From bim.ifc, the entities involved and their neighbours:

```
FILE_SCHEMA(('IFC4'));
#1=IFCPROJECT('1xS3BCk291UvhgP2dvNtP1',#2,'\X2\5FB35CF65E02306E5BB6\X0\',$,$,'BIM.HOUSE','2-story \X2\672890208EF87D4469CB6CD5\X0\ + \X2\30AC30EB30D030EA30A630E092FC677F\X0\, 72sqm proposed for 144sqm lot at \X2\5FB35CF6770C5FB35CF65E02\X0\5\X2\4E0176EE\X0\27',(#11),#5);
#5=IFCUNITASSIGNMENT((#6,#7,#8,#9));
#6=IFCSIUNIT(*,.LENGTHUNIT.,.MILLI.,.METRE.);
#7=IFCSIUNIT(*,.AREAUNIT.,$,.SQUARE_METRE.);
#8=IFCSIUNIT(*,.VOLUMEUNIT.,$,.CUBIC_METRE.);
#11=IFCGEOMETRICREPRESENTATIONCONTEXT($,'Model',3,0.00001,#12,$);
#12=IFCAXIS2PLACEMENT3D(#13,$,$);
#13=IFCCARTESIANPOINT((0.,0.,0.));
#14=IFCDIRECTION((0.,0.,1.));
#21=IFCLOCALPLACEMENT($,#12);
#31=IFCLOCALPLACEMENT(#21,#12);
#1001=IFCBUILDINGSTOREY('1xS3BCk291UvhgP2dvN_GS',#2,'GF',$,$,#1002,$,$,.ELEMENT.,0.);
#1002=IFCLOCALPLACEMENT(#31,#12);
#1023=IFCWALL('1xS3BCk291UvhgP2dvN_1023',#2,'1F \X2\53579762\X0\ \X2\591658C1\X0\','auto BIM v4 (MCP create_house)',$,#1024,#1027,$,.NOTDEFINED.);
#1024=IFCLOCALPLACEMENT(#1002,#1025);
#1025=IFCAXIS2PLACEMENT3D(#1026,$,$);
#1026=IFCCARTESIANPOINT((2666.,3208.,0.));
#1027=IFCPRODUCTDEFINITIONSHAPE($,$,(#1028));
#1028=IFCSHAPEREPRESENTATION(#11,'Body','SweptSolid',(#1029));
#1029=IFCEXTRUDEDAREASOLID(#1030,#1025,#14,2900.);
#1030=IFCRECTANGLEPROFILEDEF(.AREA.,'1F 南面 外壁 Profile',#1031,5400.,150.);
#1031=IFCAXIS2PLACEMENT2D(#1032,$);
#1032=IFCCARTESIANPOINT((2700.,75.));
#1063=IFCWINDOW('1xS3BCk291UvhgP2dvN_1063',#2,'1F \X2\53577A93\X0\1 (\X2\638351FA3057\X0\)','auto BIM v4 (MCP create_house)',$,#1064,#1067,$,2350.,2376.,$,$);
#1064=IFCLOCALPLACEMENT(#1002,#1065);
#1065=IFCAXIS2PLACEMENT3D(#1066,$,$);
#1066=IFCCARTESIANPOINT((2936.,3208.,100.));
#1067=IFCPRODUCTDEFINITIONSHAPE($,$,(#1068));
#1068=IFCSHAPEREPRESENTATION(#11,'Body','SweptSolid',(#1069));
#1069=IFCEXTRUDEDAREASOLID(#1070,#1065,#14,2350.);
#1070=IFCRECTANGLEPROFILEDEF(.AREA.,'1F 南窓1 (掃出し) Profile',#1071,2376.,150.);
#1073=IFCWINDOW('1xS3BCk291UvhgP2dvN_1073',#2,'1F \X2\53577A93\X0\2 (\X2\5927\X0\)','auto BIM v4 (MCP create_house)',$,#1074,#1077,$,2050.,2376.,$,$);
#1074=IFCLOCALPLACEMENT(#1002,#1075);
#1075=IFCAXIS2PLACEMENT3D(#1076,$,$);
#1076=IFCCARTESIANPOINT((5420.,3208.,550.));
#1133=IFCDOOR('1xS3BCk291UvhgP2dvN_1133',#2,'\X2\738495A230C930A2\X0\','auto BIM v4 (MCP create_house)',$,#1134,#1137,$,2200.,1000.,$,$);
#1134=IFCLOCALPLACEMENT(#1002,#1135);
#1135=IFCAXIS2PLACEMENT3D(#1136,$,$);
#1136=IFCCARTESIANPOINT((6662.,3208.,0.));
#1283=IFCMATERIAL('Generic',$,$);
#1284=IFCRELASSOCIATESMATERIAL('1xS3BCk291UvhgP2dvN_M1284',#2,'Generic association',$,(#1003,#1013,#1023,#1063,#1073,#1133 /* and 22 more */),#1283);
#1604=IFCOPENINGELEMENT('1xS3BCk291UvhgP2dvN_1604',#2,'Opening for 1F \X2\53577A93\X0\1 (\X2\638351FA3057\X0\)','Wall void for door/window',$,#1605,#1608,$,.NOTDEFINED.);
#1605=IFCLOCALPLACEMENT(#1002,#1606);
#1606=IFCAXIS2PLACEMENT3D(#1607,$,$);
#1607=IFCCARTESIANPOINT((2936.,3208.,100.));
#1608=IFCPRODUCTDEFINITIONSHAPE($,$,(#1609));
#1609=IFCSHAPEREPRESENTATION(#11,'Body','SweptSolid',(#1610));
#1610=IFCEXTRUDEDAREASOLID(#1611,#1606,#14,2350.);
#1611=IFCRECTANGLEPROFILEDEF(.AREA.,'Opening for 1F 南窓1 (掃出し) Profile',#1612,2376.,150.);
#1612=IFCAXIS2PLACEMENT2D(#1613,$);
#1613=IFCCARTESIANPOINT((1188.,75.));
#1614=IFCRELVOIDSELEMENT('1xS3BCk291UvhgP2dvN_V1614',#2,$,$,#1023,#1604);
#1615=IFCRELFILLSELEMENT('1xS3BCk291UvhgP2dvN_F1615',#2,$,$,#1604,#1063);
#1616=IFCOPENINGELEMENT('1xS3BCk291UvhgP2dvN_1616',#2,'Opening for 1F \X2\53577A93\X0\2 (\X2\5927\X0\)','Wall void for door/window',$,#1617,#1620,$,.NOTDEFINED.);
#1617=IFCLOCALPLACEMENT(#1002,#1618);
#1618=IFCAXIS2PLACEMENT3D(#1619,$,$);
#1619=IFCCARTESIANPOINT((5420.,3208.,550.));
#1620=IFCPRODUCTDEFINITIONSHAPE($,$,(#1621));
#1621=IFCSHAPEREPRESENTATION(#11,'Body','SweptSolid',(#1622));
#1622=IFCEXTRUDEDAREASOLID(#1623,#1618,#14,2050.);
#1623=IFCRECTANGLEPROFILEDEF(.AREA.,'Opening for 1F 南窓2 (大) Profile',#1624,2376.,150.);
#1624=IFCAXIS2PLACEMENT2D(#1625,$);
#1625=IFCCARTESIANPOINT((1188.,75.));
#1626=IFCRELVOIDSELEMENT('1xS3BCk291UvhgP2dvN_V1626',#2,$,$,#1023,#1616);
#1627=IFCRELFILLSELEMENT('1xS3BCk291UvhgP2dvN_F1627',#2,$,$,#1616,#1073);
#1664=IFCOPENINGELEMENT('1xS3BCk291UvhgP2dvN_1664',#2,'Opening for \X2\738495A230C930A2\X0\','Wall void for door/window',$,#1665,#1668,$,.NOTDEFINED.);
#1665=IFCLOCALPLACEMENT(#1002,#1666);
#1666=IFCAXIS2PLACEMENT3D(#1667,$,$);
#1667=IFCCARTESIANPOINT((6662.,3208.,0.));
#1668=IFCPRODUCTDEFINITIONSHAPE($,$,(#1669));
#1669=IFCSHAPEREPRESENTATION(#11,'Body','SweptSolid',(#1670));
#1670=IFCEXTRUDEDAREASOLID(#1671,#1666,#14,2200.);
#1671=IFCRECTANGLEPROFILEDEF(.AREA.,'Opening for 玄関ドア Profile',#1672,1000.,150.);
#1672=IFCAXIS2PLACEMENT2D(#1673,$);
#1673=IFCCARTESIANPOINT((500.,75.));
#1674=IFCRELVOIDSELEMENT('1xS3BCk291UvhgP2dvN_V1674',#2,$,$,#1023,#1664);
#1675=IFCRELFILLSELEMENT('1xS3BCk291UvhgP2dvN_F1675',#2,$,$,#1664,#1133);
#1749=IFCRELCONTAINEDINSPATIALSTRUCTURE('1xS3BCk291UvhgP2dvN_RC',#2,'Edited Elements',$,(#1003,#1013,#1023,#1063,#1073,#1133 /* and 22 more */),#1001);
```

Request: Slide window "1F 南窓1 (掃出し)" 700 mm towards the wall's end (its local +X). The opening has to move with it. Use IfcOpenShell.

```python
import ifcopenshell
import ifcopenshell.api.geometry
import ifcopenshell.util.placement
import ifcopenshell.util.unit

model = ifcopenshell.open("bim.ifc")
unit_scale = ifcopenshell.util.unit.calculate_unit_scale(model)

window = model.by_guid("1xS3BCk291UvhgP2dvN_1063")
opening = window.FillsVoids[0].RelatingOpeningElement
wall = opening.VoidsElements[0].RelatingBuildingElement

wall_matrix = ifcopenshell.util.placement.get_local_placement(wall.ObjectPlacement)
shift = wall_matrix[:3, 0] * 0.7 / unit_scale
before = ifcopenshell.util.placement.get_local_placement(window.ObjectPlacement)[:3, 3].copy()

# The window is not placed relative to its opening, so move both.
for product in (opening, window):
    matrix = ifcopenshell.util.placement.get_local_placement(product.ObjectPlacement)
    matrix[:3, 3] += shift
    ifcopenshell.api.geometry.edit_object_placement(model, product=product, matrix=matrix, is_si=False)

after = ifcopenshell.util.placement.get_local_placement(window.ObjectPlacement)[:3, 3]
print("window moved by", (after - before).round(3) + 0.0)

model.write("bim_v2.ifc")
```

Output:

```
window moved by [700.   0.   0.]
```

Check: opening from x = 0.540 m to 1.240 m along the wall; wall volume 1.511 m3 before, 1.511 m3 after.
